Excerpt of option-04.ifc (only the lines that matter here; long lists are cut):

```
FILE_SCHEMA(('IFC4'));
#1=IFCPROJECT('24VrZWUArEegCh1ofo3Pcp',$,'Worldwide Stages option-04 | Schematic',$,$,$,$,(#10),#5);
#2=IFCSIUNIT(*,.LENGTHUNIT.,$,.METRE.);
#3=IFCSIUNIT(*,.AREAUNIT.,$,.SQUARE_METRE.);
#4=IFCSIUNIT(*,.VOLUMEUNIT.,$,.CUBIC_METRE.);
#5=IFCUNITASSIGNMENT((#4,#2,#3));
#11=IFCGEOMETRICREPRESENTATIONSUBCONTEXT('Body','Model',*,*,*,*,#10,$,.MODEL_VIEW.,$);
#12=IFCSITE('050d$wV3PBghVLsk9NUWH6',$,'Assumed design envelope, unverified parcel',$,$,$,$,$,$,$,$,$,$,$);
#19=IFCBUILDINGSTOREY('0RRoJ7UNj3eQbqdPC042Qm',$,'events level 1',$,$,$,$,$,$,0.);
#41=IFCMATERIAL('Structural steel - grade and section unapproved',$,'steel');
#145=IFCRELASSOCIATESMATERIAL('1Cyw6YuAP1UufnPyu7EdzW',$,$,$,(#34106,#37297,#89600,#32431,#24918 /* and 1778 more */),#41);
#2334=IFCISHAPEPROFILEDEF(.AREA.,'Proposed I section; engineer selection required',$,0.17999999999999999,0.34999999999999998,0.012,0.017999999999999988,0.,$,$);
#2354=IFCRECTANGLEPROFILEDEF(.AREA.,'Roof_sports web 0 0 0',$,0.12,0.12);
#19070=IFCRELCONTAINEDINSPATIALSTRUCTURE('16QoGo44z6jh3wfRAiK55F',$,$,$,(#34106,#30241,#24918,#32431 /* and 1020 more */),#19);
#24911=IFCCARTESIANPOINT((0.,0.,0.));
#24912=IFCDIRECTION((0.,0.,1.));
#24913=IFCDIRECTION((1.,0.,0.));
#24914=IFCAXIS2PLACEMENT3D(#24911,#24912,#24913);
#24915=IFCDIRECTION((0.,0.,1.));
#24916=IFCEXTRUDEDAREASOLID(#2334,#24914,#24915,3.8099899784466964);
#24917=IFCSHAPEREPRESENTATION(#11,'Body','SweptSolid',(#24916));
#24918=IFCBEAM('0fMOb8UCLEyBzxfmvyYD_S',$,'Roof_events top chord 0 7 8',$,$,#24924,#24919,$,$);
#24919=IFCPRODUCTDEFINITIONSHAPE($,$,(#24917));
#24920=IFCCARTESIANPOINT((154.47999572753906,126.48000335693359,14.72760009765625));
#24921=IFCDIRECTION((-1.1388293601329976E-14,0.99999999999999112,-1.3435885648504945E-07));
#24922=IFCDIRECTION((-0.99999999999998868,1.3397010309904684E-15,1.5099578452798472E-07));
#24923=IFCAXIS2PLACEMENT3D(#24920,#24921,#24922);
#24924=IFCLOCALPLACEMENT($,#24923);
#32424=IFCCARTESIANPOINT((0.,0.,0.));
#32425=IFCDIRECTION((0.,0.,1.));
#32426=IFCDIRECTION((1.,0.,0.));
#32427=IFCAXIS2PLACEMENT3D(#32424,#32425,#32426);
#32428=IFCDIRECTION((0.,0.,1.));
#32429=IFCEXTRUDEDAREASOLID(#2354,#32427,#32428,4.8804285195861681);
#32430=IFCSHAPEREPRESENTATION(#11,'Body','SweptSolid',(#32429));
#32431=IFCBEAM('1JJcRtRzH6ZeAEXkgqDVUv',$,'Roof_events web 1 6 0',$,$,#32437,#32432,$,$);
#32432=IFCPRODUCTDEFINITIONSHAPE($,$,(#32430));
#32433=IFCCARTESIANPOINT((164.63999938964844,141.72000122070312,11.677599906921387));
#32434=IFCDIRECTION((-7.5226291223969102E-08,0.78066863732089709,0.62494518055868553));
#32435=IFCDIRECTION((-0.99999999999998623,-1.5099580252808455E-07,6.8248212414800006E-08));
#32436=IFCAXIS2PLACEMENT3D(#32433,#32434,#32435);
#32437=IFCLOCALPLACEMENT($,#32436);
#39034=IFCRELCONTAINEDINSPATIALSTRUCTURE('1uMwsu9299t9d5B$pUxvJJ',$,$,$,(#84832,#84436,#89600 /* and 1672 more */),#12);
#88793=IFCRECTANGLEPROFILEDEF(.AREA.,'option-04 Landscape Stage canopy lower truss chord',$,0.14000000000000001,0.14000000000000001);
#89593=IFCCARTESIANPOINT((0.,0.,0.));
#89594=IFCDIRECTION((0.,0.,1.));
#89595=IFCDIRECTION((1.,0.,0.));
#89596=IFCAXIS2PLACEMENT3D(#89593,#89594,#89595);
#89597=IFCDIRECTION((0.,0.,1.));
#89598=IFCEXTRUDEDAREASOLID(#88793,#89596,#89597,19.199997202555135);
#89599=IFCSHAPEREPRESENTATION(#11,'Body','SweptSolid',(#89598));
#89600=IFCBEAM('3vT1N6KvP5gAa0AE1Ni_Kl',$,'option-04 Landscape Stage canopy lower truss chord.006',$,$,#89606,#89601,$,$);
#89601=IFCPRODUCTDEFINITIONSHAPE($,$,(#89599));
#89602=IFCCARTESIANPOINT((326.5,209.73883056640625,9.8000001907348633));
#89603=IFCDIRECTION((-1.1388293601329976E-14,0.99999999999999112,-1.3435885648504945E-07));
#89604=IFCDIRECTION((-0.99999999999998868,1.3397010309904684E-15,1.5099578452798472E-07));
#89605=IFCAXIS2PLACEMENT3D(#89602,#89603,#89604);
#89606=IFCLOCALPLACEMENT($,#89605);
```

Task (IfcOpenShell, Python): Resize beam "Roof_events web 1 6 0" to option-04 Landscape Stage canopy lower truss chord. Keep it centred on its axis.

```python
import ifcopenshell
import ifcopenshell.util.element
import ifcopenshell.util.representation

model = ifcopenshell.open("option-04.ifc")

member = model.by_guid("1JJcRtRzH6ZeAEXkgqDVUv")
source = next(p for p in model.by_type("IfcRectangleProfileDef") if p.ProfileName == "option-04 Landscape Stage canopy lower truss chord")

body = ifcopenshell.util.representation.get_representation(member, "Model", "Body")
solid = body.Items[0]
old_profile = solid.SweptArea

# Copy the section's sizes but keep this member's own profile position.
profile = ifcopenshell.util.element.copy(model, source)
profile.Position = old_profile.Position
solid.SweptArea = profile
if not model.get_total_inverses(old_profile):
    ifcopenshell.util.element.remove_deep2(model, old_profile)

print(solid.SweptArea)

model.write("option-04_v2.ifc")
```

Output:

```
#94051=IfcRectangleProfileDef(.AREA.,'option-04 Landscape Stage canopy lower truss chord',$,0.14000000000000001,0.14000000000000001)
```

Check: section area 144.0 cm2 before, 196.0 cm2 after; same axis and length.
